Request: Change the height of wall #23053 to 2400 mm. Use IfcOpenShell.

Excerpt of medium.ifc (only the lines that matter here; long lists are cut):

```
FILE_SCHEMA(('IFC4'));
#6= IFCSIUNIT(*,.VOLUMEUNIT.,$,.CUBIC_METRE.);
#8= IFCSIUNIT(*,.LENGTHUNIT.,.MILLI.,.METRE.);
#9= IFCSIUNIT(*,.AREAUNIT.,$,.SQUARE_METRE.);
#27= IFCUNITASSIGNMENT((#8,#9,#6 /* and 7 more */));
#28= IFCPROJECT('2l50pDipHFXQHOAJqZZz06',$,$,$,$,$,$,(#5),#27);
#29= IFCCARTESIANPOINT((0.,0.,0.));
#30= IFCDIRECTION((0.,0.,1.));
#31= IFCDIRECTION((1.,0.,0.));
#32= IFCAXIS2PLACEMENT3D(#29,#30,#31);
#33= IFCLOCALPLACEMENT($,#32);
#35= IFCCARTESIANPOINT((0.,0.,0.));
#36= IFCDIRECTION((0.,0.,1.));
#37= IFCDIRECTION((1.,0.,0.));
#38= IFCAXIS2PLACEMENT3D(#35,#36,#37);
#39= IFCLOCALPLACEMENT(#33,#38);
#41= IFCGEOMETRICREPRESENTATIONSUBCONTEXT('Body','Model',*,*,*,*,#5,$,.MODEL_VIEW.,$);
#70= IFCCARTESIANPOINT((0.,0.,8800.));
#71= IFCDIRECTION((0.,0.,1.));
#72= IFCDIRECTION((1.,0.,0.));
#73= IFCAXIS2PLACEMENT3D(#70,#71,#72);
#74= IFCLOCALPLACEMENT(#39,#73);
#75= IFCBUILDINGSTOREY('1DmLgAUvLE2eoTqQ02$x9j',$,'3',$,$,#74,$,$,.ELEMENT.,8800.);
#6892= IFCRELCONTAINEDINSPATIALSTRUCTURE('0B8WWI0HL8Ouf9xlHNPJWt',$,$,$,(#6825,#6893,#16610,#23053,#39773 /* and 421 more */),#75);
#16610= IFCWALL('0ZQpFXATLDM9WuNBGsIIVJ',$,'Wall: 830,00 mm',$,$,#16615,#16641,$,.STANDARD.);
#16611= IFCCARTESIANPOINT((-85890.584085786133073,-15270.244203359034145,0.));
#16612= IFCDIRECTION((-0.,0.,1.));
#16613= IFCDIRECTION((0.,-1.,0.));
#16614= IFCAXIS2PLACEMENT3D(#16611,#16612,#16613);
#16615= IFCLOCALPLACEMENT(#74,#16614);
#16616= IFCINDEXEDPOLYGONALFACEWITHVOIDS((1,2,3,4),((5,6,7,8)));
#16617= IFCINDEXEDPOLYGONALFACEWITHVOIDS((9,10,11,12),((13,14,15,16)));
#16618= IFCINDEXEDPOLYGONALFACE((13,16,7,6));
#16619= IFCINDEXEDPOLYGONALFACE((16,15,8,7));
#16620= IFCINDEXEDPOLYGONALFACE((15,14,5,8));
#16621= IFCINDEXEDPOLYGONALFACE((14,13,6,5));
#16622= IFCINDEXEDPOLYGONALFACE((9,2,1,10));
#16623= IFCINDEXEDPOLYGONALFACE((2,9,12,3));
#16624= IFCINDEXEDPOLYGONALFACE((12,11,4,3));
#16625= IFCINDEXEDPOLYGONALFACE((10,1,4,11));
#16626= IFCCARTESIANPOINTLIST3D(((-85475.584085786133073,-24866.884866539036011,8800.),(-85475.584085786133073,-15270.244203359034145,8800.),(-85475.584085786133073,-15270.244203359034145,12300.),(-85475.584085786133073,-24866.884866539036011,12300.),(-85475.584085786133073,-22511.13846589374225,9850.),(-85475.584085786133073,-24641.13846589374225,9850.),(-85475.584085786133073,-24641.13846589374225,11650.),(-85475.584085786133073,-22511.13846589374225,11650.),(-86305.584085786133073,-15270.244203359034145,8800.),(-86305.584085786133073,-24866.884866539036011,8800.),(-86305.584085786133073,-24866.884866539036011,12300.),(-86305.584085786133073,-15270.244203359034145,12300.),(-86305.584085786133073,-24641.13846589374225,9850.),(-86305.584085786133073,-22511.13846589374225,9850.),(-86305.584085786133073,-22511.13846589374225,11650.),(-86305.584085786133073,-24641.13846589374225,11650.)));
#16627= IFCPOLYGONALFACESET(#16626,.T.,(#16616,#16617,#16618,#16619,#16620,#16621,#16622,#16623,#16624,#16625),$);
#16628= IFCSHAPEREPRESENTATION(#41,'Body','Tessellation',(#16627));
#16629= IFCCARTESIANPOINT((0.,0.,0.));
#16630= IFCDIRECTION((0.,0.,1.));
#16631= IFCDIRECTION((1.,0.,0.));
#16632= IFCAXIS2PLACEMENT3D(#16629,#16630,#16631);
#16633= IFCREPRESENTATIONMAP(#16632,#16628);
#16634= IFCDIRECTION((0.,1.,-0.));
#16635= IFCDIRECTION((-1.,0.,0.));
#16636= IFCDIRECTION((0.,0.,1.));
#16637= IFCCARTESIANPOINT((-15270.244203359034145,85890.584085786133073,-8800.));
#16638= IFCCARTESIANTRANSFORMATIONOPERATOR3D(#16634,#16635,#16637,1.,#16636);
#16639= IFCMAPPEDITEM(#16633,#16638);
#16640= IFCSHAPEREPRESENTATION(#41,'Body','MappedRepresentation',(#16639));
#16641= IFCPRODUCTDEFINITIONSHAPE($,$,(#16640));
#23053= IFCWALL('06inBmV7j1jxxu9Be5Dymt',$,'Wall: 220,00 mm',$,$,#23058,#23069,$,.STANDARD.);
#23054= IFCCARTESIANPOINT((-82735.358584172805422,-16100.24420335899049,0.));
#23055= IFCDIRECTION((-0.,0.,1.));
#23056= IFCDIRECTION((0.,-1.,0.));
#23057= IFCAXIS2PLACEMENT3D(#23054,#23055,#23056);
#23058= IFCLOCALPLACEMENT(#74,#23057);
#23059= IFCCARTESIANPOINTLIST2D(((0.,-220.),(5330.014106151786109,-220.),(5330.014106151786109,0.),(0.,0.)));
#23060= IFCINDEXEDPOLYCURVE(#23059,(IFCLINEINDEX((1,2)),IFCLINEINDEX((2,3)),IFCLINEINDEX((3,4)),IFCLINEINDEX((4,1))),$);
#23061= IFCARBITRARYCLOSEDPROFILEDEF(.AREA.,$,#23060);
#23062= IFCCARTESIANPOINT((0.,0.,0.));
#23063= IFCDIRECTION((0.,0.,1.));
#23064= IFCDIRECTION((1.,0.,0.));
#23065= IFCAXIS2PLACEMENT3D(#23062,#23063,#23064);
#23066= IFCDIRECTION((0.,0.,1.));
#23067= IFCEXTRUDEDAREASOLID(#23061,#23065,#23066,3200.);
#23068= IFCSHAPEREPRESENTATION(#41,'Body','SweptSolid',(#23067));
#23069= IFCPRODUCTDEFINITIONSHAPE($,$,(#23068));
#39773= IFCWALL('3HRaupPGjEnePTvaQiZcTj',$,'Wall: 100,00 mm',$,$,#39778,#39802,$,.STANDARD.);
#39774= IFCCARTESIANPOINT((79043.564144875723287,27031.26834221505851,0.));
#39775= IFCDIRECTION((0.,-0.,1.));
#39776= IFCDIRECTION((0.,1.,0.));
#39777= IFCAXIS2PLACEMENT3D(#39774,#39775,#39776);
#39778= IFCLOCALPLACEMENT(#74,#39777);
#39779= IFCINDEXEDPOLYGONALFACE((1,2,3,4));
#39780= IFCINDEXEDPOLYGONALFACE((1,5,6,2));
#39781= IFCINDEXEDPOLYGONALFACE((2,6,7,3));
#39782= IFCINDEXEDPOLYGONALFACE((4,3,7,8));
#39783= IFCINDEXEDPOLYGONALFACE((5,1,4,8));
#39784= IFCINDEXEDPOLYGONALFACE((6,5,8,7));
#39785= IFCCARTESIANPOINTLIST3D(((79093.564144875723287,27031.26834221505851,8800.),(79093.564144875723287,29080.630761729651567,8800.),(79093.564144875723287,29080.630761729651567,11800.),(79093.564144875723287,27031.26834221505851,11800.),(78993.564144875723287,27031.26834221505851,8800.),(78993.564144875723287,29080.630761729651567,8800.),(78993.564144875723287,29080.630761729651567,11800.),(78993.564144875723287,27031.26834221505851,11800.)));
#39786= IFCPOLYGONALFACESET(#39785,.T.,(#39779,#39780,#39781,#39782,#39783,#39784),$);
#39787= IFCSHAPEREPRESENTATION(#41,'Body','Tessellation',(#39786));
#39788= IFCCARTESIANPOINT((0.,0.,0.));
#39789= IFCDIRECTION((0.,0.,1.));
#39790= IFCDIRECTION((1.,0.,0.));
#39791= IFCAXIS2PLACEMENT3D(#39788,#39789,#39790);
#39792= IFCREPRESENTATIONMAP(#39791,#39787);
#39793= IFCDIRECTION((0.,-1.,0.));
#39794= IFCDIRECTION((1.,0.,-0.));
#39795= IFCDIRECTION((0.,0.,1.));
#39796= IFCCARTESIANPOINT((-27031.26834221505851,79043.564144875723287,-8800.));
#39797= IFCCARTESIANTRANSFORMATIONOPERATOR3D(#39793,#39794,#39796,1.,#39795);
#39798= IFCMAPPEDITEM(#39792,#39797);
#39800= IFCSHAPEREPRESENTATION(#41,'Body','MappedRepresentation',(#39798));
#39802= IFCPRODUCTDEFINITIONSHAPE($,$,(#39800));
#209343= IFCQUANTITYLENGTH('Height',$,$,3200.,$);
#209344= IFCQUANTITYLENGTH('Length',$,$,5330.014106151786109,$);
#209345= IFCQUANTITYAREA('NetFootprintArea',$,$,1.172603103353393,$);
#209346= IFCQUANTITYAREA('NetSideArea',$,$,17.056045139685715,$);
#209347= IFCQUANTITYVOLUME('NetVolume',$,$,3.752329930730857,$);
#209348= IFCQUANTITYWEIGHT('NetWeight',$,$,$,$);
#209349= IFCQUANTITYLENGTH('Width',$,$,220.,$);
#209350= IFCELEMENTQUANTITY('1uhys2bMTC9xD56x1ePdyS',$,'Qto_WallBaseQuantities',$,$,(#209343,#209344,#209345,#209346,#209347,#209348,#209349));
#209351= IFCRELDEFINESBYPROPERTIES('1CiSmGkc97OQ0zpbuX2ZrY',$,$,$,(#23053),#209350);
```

```python
import ifcopenshell
import ifcopenshell.api.pset
import ifcopenshell.geom
import ifcopenshell.util.element
import ifcopenshell.util.representation
import ifcopenshell.util.shape
import ifcopenshell.util.unit

model = ifcopenshell.open("medium.ifc")
area_scale = ifcopenshell.util.unit.calculate_unit_scale(model, "AREAUNIT")
volume_scale = ifcopenshell.util.unit.calculate_unit_scale(model, "VOLUMEUNIT")
settings = ifcopenshell.geom.settings()


def volume(element):
    """Net volume in cubic metres, openings subtracted."""
    shape = ifcopenshell.geom.create_shape(settings, element)
    return ifcopenshell.util.shape.get_volume(shape.geometry)


wall = model.by_id(23053)
before = volume(wall)

body = ifcopenshell.util.representation.get_representation(wall, "Model", "Body")
solid = body.Items[0]
old_height = solid.Depth
solid.Depth = 2400.0
after = volume(wall)
thickness = 0.22  # wall thickness in metres

# Update the stored height, areas and volumes.
qto = model.by_id(ifcopenshell.util.element.get_pset(wall, "Qto_WallBaseQuantities", should_inherit=False)["id"])
ifcopenshell.api.pset.edit_qto(model, qto=qto, properties={
    "Height": solid.Depth,
    "NetSideArea": after / thickness / area_scale,
    "NetVolume": after / volume_scale,
})

print(f"height {old_height:g} -> {solid.Depth:g}, volume {before:.3f} -> {after:.3f} m3")

model.write("medium_rev.ifc")
```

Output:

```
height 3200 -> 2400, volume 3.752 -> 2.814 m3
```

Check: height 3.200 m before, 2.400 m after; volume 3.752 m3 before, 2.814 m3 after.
